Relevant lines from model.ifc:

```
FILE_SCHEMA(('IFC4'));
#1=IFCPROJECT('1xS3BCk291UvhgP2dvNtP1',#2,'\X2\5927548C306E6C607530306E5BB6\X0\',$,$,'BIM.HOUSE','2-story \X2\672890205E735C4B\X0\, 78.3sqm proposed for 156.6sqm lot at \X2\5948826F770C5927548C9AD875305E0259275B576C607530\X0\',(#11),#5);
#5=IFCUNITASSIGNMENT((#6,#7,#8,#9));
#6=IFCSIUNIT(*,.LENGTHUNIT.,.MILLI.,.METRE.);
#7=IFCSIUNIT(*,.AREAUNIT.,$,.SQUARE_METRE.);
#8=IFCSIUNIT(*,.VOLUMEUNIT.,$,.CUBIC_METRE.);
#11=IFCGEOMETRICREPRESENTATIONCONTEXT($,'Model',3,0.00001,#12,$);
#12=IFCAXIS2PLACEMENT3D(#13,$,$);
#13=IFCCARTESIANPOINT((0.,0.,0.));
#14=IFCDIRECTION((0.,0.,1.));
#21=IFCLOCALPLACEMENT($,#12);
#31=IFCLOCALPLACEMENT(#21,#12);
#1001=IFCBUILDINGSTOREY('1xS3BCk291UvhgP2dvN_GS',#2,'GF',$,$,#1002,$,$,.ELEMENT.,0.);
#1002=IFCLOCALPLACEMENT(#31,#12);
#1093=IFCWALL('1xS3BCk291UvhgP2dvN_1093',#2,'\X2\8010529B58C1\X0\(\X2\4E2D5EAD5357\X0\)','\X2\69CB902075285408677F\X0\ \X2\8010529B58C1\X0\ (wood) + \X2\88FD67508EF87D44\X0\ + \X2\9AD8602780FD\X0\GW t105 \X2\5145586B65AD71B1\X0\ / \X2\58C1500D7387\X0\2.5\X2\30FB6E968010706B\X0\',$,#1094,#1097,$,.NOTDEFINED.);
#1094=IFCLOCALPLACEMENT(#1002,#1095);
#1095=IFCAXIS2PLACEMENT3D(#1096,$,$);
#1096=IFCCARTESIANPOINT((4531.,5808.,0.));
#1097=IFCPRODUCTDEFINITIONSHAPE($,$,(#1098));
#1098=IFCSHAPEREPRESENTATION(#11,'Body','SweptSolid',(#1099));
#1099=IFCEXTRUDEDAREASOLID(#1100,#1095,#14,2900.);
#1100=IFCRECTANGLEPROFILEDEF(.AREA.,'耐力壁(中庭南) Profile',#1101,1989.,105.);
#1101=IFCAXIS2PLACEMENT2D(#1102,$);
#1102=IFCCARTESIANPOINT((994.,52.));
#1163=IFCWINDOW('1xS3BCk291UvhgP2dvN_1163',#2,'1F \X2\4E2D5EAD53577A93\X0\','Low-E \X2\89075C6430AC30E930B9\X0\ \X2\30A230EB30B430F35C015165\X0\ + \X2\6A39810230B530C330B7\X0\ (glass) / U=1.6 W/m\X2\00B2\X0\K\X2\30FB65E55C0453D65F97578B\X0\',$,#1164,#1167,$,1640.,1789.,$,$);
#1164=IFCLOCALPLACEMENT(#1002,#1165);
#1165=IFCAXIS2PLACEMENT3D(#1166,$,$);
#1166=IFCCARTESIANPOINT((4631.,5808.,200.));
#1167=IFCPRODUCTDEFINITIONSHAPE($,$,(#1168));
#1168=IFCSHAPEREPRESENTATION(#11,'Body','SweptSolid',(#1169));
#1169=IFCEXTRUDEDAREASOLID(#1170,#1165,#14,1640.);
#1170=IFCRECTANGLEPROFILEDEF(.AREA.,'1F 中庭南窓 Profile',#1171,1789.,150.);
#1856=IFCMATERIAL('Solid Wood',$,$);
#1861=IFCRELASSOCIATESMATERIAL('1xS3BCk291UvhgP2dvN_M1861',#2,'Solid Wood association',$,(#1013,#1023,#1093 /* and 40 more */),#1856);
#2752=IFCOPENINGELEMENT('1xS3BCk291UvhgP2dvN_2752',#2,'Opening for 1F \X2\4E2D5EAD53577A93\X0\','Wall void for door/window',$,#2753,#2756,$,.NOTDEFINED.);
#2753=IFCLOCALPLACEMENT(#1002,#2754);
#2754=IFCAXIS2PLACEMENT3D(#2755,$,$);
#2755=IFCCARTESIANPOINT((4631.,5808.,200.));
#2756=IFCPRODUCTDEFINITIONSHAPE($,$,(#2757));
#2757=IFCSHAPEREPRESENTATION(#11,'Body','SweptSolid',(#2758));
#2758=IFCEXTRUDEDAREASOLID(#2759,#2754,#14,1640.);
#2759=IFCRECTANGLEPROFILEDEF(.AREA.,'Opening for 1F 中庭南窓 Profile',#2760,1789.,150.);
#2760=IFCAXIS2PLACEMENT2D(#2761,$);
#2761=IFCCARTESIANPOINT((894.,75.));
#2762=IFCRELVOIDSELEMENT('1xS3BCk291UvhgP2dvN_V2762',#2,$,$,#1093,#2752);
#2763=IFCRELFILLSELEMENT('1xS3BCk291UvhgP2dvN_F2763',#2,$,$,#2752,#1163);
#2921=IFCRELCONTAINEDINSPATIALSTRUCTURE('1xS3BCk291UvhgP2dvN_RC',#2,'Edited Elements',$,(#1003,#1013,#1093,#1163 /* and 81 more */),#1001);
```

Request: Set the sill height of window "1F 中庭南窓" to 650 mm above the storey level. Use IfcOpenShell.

```python
import numpy as np
import ifcopenshell
import ifcopenshell.api.geometry
import ifcopenshell.geom
import ifcopenshell.util.element
import ifcopenshell.util.placement
import ifcopenshell.util.shape
import ifcopenshell.util.unit

model = ifcopenshell.open("model.ifc")
unit_scale = ifcopenshell.util.unit.calculate_unit_scale(model)

window = model.by_id(1163)
opening = window.FillsVoids[0].RelatingOpeningElement
storey = ifcopenshell.util.element.get_container(window, ifc_class="IfcBuildingStorey")
level = ifcopenshell.util.placement.get_local_placement(storey.ObjectPlacement)[2, 3]

# The opening's origin need not be at the sill, so measure its lowest point.
shape = ifcopenshell.geom.create_shape(ifcopenshell.geom.settings(), opening)
bottom = ifcopenshell.util.shape.get_shape_bottom_elevation(shape, shape.geometry) / unit_scale
dz = level + 0.65 / unit_scale - bottom

shift = np.array([0.0, 0.0, dz])
# The window is not placed relative to its opening, so move both.
for product in (opening, window):
    matrix = ifcopenshell.util.placement.get_local_placement(product.ObjectPlacement)
    matrix[:3, 3] += shift
    ifcopenshell.api.geometry.edit_object_placement(model, product=product, matrix=matrix, is_si=False)

print(f"moved by {dz * unit_scale:+.3f} m")

model.write("model_rev.ifc")
```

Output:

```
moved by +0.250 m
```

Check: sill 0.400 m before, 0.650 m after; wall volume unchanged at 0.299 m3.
